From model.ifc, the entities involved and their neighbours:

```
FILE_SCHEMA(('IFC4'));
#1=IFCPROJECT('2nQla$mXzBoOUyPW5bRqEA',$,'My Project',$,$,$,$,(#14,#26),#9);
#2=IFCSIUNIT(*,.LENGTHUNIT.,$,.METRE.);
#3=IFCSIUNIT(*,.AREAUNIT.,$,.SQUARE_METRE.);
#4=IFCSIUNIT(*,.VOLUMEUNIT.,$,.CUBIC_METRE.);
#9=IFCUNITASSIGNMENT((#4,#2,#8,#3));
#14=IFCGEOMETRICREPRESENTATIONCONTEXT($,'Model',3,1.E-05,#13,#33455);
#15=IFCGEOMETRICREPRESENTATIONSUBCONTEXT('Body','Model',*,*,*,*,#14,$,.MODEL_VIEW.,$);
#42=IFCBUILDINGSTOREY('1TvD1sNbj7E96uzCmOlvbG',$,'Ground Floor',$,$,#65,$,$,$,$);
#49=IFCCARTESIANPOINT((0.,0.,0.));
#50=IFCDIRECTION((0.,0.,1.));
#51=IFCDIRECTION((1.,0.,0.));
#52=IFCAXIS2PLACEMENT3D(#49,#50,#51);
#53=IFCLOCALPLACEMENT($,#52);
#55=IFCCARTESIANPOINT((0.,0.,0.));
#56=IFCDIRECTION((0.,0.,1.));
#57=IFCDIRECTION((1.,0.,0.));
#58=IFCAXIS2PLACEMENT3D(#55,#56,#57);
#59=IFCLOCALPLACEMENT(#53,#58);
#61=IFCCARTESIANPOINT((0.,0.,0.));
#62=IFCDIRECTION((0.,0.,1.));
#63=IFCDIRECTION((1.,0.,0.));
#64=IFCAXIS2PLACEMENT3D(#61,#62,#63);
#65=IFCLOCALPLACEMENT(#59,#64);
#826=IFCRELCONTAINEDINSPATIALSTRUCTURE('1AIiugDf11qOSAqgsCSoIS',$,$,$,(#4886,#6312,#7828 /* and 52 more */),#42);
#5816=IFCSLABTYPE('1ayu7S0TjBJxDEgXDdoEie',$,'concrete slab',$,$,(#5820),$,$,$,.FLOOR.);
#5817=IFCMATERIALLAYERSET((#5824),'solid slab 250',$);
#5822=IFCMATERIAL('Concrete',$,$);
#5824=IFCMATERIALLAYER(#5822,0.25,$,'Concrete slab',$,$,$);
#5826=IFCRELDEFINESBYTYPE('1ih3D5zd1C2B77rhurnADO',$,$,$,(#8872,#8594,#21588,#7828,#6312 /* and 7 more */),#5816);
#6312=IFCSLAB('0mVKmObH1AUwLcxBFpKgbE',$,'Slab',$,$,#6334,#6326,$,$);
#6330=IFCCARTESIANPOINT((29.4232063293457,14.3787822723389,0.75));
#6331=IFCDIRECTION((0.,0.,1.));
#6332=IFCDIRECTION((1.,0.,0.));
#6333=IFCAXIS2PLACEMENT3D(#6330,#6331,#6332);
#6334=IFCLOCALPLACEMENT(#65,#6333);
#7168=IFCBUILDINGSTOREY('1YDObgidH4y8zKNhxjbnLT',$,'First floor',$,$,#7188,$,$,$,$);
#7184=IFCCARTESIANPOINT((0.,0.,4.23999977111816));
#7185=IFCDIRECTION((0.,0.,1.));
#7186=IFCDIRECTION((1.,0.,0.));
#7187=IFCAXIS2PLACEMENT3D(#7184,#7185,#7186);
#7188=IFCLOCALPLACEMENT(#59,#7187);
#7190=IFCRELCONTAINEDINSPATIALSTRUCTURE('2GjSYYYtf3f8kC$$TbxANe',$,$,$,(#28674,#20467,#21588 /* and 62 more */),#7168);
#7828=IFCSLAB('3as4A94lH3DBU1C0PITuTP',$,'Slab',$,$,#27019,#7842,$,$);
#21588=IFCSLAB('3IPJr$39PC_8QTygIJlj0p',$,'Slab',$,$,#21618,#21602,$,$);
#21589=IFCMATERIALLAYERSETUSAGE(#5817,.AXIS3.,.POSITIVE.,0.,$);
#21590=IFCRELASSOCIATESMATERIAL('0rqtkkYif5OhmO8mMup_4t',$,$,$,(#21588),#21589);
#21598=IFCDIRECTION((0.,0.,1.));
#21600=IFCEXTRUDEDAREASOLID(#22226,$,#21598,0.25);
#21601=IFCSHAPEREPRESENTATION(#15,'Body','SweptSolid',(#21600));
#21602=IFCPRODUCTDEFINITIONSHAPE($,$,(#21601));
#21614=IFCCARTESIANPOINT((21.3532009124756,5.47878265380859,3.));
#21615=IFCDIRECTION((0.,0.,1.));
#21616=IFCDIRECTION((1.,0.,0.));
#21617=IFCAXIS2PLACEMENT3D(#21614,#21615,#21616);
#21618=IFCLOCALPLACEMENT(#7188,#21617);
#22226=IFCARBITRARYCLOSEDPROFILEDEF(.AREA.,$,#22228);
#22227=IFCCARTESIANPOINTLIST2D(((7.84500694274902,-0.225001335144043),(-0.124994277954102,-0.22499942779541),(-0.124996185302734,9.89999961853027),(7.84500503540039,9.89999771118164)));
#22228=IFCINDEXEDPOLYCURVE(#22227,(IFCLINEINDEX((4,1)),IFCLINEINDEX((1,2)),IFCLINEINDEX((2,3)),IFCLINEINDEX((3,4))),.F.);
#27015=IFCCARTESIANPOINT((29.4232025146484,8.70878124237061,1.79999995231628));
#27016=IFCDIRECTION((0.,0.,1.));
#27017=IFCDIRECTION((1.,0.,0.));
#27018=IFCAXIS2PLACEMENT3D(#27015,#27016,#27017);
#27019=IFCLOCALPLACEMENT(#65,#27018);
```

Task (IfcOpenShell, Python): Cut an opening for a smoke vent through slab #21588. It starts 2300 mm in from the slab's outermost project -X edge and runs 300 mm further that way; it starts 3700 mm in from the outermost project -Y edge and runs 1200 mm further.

```python
import numpy as np
import ifcopenshell
import ifcopenshell.api.feature
import ifcopenshell.api.geometry
import ifcopenshell.api.root
import ifcopenshell.geom
import ifcopenshell.util.placement
import ifcopenshell.util.representation
import ifcopenshell.util.shape
import ifcopenshell.util.unit

model = ifcopenshell.open("model.ifc")
unit_scale = ifcopenshell.util.unit.calculate_unit_scale(model)
settings = ifcopenshell.geom.settings()


def volume(element):
    """Net volume in cubic metres, openings subtracted."""
    shape = ifcopenshell.geom.create_shape(settings, element)
    return ifcopenshell.util.shape.get_volume(shape.geometry)


slab = model.by_guid("3IPJr$39PC_8QTygIJlj0p")
before = volume(slab)

# Extent in the slab's own axes, in metres. The edges named are its -X and -Y sides.
slab_shape = ifcopenshell.geom.create_shape(settings, slab)
vertices = ifcopenshell.util.shape.get_vertices(slab_shape.geometry)
x_min, y_min, bottom = vertices.min(axis=0)
top = vertices[:, 2].max()

opening = ifcopenshell.api.root.create_entity(model, ifc_class="IfcOpeningElement", name="Smoke vent opening", predefined_type="OPENING")
context = ifcopenshell.util.representation.get_context(model, "Model", "Body", "MODEL_VIEW")
width, depth = 0.3, 1.2
outline = [(0.0, 0.0), (width, 0.0), (width, depth), (0.0, depth), (0.0, 0.0)]
# Overshoot both faces by 50 mm so the cut is clean.
shape = ifcopenshell.api.geometry.add_slab_representation(
    model, context=context, depth=top - bottom + 0.1, polyline=outline
)
ifcopenshell.api.geometry.assign_representation(model, product=opening, representation=shape)

matrix = ifcopenshell.util.placement.get_local_placement(slab.ObjectPlacement)
matrix[:, 3] = matrix @ np.append(np.array([x_min + 2.3, y_min + 3.7, bottom - 0.05]) / unit_scale, 1.0)
ifcopenshell.api.geometry.edit_object_placement(model, product=opening, matrix=matrix, is_si=False)
ifcopenshell.api.feature.add_feature(model, feature=opening, element=slab)

after = volume(slab)

print(f"slab volume {before:.3f} -> {after:.3f} m3")

model.write("model-out.ifc")
```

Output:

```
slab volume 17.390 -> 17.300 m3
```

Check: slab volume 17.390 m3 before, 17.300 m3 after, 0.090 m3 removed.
